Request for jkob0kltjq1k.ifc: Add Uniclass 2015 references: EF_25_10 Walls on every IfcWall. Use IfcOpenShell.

First a look at what the model holds.

```python
import ifcopenshell

model = ifcopenshell.open("jkob0kltjq1k.ifc")
print(model.schema)
print("classifications:", [c.Name for c in model.by_type("IfcClassification")])
for ifc_class in ("IfcDoor", "IfcRoof", "IfcStair", "IfcWall", "IfcWindow"):
    print(ifc_class, len(model.by_type(ifc_class)))
```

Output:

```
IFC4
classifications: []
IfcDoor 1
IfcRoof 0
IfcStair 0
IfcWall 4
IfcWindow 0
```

```python
import ifcopenshell
import ifcopenshell.api.classification

model = ifcopenshell.open("jkob0kltjq1k.ifc")

system = ifcopenshell.api.classification.add_classification(model, classification="Uniclass 2015")

codes = {
    "IfcWall": ("EF_25_10", "Walls"),
}
for ifc_class, (code, name) in codes.items():
    products = model.by_type(ifc_class)
    ifcopenshell.api.classification.add_reference(
        model, products=products, classification=system, identification=code, name=name
    )
    print(code, len(products))

model.write("jkob0kltjq1k_rev.ifc")
```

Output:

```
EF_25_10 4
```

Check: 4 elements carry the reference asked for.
